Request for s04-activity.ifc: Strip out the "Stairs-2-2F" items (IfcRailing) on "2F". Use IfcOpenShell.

First a look at what the model holds.

```python
import ifcopenshell
import ifcopenshell.util.element

model = ifcopenshell.open("s04-activity.ifc")
print(model.schema)
storey = next(s for s in model.by_type("IfcBuildingStorey") if s.Name == "2F")
railings = [e for e in ifcopenshell.util.element.get_decomposition(storey) if e.is_a("IfcRailing")]
seen = {}
for e in railings:
    element_type = ifcopenshell.util.element.get_type(e)
    name = element_type.Name if element_type not in (None, e) else None
    seen[name] = seen.get(name, 0) + 1
for name, count in sorted(seen.items(), key=str):
    print(count, "x", name)
```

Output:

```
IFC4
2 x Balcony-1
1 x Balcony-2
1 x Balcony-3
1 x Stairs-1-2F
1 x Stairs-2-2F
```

```python
import ifcopenshell
import ifcopenshell.api.root
import ifcopenshell.util.element

model = ifcopenshell.open("s04-activity.ifc")

storey = next(s for s in model.by_type("IfcBuildingStorey") if s.Name == "2F")
railings = [e for e in ifcopenshell.util.element.get_decomposition(storey) if e.is_a("IfcRailing")]
targets = [e for e in railings if (t := ifcopenshell.util.element.get_type(e)) not in (None, e) and t.Name == "Stairs-2-2F"]

for e in targets:
    ifcopenshell.api.root.remove_product(model, product=e)
print(len(targets), "removed")

model.write("s04-activity_edited.ifc")
```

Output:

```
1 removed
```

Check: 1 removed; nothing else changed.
